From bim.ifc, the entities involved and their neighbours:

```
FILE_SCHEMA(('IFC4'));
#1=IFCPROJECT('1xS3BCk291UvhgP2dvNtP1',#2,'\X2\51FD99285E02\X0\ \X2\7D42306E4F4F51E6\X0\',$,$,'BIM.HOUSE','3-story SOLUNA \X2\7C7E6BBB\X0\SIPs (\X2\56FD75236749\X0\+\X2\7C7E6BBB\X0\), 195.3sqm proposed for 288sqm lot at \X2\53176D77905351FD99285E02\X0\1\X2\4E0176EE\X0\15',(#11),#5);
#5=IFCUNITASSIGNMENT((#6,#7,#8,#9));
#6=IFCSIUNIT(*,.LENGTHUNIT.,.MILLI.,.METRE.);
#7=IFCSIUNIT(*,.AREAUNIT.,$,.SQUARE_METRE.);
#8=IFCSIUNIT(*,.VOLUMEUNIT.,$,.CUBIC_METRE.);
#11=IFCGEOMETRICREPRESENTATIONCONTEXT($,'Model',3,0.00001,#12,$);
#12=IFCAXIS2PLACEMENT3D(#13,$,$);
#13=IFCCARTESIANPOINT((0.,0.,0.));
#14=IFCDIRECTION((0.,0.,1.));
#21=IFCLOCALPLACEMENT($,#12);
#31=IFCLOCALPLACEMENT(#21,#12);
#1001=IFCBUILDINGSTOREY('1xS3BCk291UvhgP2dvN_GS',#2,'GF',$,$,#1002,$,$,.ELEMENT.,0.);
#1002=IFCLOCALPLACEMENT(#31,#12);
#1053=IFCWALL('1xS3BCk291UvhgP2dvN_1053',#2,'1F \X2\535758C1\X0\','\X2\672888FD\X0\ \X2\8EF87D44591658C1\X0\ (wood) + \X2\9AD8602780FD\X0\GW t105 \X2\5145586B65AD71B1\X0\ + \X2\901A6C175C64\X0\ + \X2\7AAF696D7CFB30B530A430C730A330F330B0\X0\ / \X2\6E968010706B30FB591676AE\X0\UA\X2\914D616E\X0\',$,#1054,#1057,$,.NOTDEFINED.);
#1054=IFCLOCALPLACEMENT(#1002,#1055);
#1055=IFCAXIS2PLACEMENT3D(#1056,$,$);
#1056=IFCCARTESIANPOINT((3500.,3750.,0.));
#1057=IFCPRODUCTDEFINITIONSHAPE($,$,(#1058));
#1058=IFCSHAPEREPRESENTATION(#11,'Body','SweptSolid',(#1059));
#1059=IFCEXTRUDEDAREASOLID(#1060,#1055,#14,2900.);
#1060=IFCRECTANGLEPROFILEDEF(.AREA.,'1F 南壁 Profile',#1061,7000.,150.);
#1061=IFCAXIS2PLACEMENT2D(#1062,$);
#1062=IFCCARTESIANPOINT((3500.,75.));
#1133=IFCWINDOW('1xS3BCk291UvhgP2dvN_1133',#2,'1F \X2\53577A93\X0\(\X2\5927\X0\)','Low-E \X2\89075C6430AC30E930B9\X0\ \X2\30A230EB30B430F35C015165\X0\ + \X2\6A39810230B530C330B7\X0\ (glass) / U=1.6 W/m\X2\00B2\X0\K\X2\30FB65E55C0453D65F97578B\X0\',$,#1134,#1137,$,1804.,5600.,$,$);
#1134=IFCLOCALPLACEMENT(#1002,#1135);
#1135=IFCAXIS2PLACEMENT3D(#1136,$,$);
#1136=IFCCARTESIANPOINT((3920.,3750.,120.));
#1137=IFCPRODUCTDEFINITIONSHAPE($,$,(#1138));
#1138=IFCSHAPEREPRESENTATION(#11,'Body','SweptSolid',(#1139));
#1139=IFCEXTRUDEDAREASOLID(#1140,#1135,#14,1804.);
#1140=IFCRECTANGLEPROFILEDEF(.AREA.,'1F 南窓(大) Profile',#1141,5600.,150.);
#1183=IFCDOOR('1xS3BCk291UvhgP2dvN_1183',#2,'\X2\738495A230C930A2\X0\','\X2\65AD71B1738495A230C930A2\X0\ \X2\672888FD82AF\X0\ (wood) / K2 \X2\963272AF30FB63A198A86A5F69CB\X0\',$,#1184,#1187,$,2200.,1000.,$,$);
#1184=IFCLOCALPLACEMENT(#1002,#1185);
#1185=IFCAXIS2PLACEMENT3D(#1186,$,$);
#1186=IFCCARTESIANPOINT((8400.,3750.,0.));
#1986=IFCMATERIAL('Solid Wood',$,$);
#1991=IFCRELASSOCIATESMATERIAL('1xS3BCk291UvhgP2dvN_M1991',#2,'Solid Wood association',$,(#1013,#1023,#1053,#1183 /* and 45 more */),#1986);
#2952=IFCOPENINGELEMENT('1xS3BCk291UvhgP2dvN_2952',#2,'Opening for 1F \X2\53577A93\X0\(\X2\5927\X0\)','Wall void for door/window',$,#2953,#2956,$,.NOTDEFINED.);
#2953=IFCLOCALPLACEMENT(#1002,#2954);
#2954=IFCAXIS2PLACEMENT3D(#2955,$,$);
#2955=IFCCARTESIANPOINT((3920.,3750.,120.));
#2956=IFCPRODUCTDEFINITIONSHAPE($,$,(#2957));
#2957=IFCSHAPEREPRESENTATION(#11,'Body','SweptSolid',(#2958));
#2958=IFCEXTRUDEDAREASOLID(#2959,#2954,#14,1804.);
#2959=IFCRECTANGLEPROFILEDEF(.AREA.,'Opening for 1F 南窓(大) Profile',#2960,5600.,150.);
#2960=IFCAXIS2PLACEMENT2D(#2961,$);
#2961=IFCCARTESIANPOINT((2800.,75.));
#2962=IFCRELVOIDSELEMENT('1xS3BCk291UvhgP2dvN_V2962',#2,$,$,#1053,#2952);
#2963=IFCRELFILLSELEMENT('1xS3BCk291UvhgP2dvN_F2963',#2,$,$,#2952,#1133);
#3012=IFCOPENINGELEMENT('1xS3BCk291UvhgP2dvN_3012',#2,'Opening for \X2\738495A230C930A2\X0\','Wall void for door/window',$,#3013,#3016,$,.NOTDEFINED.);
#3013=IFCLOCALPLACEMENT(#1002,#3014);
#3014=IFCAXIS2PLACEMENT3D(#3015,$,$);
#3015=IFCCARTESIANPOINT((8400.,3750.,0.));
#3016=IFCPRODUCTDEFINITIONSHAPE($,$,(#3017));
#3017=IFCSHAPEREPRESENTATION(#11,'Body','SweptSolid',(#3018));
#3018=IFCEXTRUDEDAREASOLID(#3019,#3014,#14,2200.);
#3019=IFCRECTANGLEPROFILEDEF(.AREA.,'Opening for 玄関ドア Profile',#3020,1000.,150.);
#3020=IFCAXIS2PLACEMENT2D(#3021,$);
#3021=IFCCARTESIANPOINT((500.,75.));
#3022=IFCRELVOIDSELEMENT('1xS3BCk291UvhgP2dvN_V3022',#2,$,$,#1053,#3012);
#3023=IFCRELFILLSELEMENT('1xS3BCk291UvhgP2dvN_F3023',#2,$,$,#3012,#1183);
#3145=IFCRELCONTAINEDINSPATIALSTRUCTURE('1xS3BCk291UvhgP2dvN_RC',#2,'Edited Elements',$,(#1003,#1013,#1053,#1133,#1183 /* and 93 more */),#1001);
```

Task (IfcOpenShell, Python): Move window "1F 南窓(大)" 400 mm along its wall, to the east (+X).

```python
import ifcopenshell
import ifcopenshell.api.geometry
import ifcopenshell.util.placement

model = ifcopenshell.open("bim.ifc")

window = model.by_guid("1xS3BCk291UvhgP2dvN_1133")
opening = window.FillsVoids[0].RelatingOpeningElement
wall = opening.VoidsElements[0].RelatingBuildingElement

wall_matrix = ifcopenshell.util.placement.get_local_placement(wall.ObjectPlacement)
shift = wall_matrix[:3, 0] * 400.0
before = ifcopenshell.util.placement.get_local_placement(window.ObjectPlacement)[:3, 3].copy()

# The window is not placed relative to its opening, so move both.
for product in (opening, window):
    matrix = ifcopenshell.util.placement.get_local_placement(product.ObjectPlacement)
    matrix[:3, 3] += shift
    ifcopenshell.api.geometry.edit_object_placement(model, product=product, matrix=matrix, is_si=False)

after = ifcopenshell.util.placement.get_local_placement(window.ObjectPlacement)[:3, 3]
print("window moved by", (after - before).round(3) + 0.0)

model.write("bim_edited.ifc")
```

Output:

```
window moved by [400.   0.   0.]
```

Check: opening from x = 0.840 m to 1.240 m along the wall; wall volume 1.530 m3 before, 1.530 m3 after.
